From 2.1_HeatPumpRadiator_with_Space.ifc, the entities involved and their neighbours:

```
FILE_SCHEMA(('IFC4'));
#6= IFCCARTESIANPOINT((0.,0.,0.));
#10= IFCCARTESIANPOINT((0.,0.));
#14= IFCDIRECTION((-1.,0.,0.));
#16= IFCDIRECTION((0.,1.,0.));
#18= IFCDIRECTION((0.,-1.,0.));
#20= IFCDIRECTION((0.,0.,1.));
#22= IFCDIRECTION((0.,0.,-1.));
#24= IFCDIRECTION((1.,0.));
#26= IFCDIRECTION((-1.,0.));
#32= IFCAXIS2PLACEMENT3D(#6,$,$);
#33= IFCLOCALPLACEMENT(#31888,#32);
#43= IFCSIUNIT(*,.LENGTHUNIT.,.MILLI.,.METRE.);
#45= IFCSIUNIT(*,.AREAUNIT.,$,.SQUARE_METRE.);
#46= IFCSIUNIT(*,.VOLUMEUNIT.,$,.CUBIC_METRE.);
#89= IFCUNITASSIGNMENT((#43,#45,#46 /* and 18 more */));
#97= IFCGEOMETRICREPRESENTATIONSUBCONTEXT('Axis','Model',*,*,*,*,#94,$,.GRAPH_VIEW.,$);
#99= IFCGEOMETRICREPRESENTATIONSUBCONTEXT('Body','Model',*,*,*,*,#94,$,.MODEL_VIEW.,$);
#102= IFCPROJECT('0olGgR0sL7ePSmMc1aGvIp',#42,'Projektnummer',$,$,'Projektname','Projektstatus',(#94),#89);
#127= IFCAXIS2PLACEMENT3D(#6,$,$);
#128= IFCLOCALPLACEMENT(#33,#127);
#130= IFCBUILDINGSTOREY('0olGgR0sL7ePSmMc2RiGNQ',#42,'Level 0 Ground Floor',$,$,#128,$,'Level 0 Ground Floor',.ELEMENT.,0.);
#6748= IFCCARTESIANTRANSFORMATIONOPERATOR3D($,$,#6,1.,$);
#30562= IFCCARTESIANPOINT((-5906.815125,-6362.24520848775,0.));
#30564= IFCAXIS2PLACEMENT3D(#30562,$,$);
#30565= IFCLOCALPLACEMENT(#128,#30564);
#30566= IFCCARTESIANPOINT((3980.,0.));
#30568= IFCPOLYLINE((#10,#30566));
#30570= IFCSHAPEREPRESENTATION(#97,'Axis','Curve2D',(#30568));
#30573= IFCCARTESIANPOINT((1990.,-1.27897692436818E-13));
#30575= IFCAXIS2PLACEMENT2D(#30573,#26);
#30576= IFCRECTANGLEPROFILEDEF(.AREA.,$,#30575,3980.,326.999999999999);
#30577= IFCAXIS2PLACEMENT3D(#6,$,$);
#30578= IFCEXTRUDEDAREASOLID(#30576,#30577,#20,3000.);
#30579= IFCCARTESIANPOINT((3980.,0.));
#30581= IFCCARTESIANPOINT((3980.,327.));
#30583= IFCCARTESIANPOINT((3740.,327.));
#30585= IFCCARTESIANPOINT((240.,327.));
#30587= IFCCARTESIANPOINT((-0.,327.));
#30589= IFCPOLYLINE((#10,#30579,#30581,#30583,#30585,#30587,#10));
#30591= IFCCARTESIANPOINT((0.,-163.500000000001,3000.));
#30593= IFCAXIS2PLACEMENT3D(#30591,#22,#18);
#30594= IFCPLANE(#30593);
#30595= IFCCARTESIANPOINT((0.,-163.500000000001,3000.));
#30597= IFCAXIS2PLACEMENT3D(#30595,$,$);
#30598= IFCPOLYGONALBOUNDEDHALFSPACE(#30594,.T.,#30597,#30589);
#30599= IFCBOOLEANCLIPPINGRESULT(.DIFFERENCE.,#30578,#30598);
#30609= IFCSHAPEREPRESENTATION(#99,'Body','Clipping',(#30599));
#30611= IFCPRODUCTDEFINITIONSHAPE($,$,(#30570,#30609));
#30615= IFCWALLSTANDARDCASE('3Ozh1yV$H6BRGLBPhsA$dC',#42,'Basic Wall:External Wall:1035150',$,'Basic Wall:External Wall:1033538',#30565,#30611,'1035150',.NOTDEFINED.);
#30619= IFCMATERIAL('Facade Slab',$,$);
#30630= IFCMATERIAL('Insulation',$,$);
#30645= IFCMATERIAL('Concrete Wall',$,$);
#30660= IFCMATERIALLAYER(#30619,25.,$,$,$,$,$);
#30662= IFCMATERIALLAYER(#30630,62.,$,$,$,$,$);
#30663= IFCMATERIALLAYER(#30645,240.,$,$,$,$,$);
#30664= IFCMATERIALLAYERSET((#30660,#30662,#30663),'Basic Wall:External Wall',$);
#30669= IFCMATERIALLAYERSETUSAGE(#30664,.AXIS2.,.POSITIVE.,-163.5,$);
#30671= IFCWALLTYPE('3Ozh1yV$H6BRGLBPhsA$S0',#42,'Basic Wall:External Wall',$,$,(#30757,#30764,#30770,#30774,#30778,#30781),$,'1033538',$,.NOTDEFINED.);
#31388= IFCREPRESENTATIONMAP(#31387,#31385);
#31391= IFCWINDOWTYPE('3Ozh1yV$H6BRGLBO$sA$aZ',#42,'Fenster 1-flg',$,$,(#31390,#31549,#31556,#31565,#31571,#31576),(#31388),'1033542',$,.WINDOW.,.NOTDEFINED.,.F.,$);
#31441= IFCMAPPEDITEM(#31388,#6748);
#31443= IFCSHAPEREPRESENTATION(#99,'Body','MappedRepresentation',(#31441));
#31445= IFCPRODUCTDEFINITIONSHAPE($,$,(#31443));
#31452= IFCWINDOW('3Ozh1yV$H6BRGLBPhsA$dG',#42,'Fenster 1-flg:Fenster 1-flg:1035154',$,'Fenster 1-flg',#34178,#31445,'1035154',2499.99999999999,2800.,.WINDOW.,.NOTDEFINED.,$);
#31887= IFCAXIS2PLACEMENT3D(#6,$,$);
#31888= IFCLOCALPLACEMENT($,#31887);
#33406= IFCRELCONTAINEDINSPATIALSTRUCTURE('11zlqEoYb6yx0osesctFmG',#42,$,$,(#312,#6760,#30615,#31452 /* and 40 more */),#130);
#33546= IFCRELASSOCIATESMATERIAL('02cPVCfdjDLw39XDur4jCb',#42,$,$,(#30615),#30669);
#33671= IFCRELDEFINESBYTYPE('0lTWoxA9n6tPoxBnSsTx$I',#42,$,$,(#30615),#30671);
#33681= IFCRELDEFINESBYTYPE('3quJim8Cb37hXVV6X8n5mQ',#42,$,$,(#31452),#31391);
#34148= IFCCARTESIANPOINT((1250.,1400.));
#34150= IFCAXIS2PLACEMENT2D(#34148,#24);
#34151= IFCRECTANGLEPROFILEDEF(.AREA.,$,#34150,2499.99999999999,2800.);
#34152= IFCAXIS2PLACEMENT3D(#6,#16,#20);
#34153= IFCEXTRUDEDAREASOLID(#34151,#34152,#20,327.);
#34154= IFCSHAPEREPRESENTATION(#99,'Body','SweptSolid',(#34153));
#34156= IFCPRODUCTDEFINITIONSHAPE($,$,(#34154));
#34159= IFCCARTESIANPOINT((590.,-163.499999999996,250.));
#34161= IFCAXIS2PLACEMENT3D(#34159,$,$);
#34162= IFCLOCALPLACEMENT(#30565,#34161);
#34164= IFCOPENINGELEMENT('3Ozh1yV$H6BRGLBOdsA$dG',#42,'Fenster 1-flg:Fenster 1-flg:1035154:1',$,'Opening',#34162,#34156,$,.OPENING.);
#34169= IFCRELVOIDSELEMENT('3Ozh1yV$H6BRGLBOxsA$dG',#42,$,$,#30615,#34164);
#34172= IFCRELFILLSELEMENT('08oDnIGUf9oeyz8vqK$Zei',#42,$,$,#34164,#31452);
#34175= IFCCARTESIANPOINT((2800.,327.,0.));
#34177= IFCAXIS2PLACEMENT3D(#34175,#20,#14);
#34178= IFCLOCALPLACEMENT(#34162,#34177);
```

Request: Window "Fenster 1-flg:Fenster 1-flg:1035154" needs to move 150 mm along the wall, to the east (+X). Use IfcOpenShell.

```python
import ifcopenshell
import ifcopenshell.api.geometry
import ifcopenshell.util.placement

model = ifcopenshell.open("2.1_HeatPumpRadiator_with_Space.ifc")

window = model.by_guid("3Ozh1yV$H6BRGLBPhsA$dG")
opening = window.FillsVoids[0].RelatingOpeningElement
wall = opening.VoidsElements[0].RelatingBuildingElement

wall_matrix = ifcopenshell.util.placement.get_local_placement(wall.ObjectPlacement)
shift = wall_matrix[:3, 0] * 150.0
before = ifcopenshell.util.placement.get_local_placement(window.ObjectPlacement)[:3, 3].copy()

# The window is placed relative to its opening, so it follows when the opening moves.
matrix = ifcopenshell.util.placement.get_local_placement(opening.ObjectPlacement)
matrix[:3, 3] += shift
ifcopenshell.api.geometry.edit_object_placement(
    model, product=opening, matrix=matrix, is_si=False, should_transform_children=True
)

after = ifcopenshell.util.placement.get_local_placement(window.ObjectPlacement)[:3, 3]
print("window moved by", (after - before).round(3) + 0.0)

model.write("2.1_HeatPumpRadiator_with_Space_edited.ifc")
```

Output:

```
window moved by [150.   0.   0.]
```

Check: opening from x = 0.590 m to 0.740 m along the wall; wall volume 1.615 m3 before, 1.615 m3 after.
